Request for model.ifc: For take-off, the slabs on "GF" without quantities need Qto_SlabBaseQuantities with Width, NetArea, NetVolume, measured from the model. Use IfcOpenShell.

First a look at what the model holds.

```python
import ifcopenshell
import ifcopenshell.util.element
import ifcopenshell.util.unit

model = ifcopenshell.open("model.ifc")
print(model.schema)
for unit_type in ("LENGTHUNIT", "AREAUNIT", "VOLUMEUNIT"):
    print(unit_type, ifcopenshell.util.unit.calculate_unit_scale(model, unit_type))
storey = next(s for s in model.by_type("IfcBuildingStorey") if s.Name == "GF")
slabs = [e for e in ifcopenshell.util.element.get_decomposition(storey) if e.is_a("IfcSlab")]
for e in sorted(slabs, key=lambda e: e.id()):
    print(e.id(), e.is_a(), e.Name, list(ifcopenshell.util.element.get_psets(e, qtos_only=True)), sep=" | ")
```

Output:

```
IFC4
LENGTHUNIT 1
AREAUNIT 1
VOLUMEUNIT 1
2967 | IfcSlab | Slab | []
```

```python
import ifcopenshell
import ifcopenshell.api.pset
import ifcopenshell.geom
import ifcopenshell.util.element
import ifcopenshell.util.shape
import ifcopenshell.util.unit

model = ifcopenshell.open("model.ifc")
unit_scale = ifcopenshell.util.unit.calculate_unit_scale(model)
area_scale = ifcopenshell.util.unit.calculate_unit_scale(model, "AREAUNIT")
volume_scale = ifcopenshell.util.unit.calculate_unit_scale(model, "VOLUMEUNIT")
settings = ifcopenshell.geom.settings()

storey = next(s for s in model.by_type("IfcBuildingStorey") if s.Name == "GF")
slabs = [e for e in ifcopenshell.util.element.get_decomposition(storey) if e.is_a("IfcSlab")]

for e in sorted(slabs, key=lambda e: e.id()):
    if ifcopenshell.util.element.get_psets(e, qtos_only=True, should_inherit=False):
        continue
    # Geometry comes back in metres, in the element's own axes.
    shape = ifcopenshell.geom.create_shape(settings, e)
    values = {
        "Width": ifcopenshell.util.shape.get_z(shape.geometry) / unit_scale,
        "NetArea": ifcopenshell.util.shape.get_footprint_area(shape.geometry) / area_scale,
        "NetVolume": ifcopenshell.util.shape.get_volume(shape.geometry) / volume_scale,
    }
    qto = ifcopenshell.api.pset.add_qto(model, product=e, name="Qto_SlabBaseQuantities")
    ifcopenshell.api.pset.edit_qto(model, qto=qto, properties=values)
    print(e.id(), {k: round(v, 3) for k, v in values.items()})

model.write("model-out.ifc")
```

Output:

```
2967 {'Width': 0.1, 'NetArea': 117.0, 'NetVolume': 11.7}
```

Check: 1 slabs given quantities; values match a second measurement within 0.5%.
